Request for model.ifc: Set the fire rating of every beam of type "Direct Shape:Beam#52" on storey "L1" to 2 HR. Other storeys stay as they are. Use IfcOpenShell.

First a look at what the model holds.

```python
import ifcopenshell
import ifcopenshell.util.element

model = ifcopenshell.open("model.ifc")
print(model.schema)
storey = next(s for s in model.by_type("IfcBuildingStorey") if s.Name == "L1")
beams = [e for e in ifcopenshell.util.element.get_decomposition(storey) if e.is_a("IfcBeam")]
seen = {}
for e in beams:
    element_type = ifcopenshell.util.element.get_type(e)
    key = (element_type.Name if element_type != e and element_type else None, ifcopenshell.util.element.get_pset(e, "Pset_BeamCommon", "FireRating"))
    seen[key] = seen.get(key, 0) + 1
for (name, value), count in sorted(seen.items(), key=str):
    print(count, "x", name, "|", value)
```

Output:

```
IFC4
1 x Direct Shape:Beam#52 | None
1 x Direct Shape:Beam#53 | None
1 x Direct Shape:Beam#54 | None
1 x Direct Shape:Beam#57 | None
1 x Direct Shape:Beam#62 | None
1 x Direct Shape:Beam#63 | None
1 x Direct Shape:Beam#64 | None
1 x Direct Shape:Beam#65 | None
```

```python
import ifcopenshell
import ifcopenshell.api.pset
import ifcopenshell.util.element

model = ifcopenshell.open("model.ifc")

storey = next(s for s in model.by_type("IfcBuildingStorey") if s.Name == "L1")
beams = [e for e in ifcopenshell.util.element.get_decomposition(storey) if e.is_a("IfcBeam")]

count = 0
for e in beams:
    element_type = ifcopenshell.util.element.get_type(e)
    if element_type in (None, e) or element_type.Name != "Direct Shape:Beam#52":
        continue
    # add_pset returns the element's existing set when there is one.
    pset = ifcopenshell.api.pset.add_pset(model, product=e, name="Pset_BeamCommon")
    ifcopenshell.api.pset.edit_pset(model, pset=pset, properties={"FireRating": "2 HR"})
    count += 1

print(count, "beams updated")

model.write("model-out.ifc")
```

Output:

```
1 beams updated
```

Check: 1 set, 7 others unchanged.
